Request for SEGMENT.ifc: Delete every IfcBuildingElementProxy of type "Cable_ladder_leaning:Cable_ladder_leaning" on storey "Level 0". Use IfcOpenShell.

First a look at what the model holds.

```python
import ifcopenshell
import ifcopenshell.util.element

model = ifcopenshell.open("SEGMENT.ifc")
print(model.schema)
storey = next(s for s in model.by_type("IfcBuildingStorey") if s.Name == "Level 0")
proxies = [e for e in ifcopenshell.util.element.get_decomposition(storey) if e.is_a("IfcBuildingElementProxy")]
seen = {}
for e in proxies:
    element_type = ifcopenshell.util.element.get_type(e)
    name = element_type.Name if element_type not in (None, e) else None
    seen[name] = seen.get(name, 0) + 1
for name, count in sorted(seen.items(), key=str):
    print(count, "x", name)
```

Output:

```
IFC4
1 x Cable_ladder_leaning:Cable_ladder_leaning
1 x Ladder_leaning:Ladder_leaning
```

```python
import ifcopenshell
import ifcopenshell.api.root
import ifcopenshell.util.element

model = ifcopenshell.open("SEGMENT.ifc")

storey = next(s for s in model.by_type("IfcBuildingStorey") if s.Name == "Level 0")
proxies = [e for e in ifcopenshell.util.element.get_decomposition(storey) if e.is_a("IfcBuildingElementProxy")]
targets = [e for e in proxies if (t := ifcopenshell.util.element.get_type(e)) not in (None, e) and t.Name == "Cable_ladder_leaning:Cable_ladder_leaning"]

for e in targets:
    ifcopenshell.api.root.remove_product(model, product=e)
print(len(targets), "removed")

model.write("SEGMENT_updated.ifc")
```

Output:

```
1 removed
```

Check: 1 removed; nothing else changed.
